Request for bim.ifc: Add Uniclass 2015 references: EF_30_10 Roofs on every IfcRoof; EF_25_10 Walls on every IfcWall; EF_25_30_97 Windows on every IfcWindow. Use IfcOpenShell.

First a look at what the model holds.

```python
import ifcopenshell

model = ifcopenshell.open("bim.ifc")
print(model.schema)
print("classifications:", [c.Name for c in model.by_type("IfcClassification")])
for ifc_class in ("IfcDoor", "IfcRoof", "IfcStair", "IfcWall", "IfcWindow"):
    print(ifc_class, len(model.by_type(ifc_class)))
```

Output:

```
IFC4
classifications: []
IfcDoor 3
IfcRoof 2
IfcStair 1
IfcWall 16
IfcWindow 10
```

```python
import ifcopenshell
import ifcopenshell.api.classification

model = ifcopenshell.open("bim.ifc")

system = ifcopenshell.api.classification.add_classification(model, classification="Uniclass 2015")

codes = {
    "IfcRoof": ("EF_30_10", "Roofs"),
    "IfcWall": ("EF_25_10", "Walls"),
    "IfcWindow": ("EF_25_30_97", "Windows"),
}
for ifc_class, (code, name) in codes.items():
    products = model.by_type(ifc_class)
    ifcopenshell.api.classification.add_reference(
        model, products=products, classification=system, identification=code, name=name
    )
    print(code, len(products))

model.write("bim_edited.ifc")
```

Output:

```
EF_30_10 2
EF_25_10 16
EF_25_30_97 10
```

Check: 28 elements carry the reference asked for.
